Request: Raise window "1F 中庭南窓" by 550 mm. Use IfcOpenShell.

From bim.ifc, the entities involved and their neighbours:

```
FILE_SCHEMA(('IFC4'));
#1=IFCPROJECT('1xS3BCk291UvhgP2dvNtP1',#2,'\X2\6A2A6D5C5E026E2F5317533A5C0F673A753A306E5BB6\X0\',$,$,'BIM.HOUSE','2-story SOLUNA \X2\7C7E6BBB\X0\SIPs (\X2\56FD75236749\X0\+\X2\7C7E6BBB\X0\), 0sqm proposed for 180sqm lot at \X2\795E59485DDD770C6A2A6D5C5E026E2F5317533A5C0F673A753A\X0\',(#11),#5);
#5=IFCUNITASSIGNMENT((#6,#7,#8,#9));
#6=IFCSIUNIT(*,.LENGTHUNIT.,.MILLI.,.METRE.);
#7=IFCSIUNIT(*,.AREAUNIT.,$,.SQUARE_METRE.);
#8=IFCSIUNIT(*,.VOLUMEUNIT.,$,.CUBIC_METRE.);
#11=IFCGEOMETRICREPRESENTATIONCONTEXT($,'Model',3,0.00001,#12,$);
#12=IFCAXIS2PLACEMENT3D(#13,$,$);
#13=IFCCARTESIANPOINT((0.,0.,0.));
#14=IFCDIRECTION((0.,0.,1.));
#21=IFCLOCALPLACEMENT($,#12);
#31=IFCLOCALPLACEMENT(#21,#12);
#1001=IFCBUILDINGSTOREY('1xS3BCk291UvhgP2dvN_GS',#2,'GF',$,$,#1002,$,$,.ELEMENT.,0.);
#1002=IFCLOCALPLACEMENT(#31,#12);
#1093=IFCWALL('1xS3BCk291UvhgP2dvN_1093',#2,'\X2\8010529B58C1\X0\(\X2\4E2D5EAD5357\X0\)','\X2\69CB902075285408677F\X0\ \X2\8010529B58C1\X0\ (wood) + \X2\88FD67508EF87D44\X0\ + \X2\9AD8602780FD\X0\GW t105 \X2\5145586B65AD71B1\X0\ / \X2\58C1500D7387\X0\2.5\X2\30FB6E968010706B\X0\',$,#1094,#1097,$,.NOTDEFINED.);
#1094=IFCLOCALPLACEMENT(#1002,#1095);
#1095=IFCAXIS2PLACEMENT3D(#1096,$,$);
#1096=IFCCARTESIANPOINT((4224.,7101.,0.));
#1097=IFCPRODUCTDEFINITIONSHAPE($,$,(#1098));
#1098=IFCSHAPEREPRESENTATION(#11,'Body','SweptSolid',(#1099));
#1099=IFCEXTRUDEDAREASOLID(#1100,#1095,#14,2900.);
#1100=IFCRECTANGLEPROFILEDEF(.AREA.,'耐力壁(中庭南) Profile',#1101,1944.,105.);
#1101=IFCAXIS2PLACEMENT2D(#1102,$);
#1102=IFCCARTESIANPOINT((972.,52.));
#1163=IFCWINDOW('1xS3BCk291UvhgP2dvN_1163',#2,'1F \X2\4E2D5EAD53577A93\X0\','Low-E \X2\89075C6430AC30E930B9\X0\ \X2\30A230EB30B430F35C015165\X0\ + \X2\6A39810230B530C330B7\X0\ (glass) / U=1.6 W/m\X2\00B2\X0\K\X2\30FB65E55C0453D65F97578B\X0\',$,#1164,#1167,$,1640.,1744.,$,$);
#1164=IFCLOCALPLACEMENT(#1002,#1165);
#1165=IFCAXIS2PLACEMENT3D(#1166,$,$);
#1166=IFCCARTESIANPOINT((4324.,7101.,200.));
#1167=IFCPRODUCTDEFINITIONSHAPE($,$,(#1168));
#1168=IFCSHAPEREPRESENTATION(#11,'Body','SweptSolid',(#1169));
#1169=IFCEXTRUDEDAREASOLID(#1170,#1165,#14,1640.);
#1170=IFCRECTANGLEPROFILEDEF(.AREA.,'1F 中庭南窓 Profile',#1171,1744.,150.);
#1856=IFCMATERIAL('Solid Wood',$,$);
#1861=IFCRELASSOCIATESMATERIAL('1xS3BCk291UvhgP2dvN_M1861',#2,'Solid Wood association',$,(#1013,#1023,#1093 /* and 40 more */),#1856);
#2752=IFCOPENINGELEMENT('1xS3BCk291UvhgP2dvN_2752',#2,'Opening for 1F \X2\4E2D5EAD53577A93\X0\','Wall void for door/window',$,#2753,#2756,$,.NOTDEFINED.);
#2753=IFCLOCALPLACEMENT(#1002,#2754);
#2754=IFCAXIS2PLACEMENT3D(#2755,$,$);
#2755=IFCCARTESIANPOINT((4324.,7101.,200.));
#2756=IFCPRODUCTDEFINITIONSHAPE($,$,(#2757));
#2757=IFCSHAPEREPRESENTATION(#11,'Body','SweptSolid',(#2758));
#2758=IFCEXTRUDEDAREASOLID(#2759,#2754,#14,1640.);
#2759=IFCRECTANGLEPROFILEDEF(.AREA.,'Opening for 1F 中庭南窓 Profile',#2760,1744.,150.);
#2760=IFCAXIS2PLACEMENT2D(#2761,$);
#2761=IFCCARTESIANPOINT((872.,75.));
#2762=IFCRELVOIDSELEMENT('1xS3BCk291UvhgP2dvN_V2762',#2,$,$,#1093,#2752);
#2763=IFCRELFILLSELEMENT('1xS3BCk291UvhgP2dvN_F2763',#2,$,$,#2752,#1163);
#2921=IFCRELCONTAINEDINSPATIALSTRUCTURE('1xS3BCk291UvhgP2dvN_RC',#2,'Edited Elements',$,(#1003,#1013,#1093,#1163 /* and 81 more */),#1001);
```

```python
import numpy as np
import ifcopenshell
import ifcopenshell.api.geometry
import ifcopenshell.util.placement
import ifcopenshell.util.unit

model = ifcopenshell.open("bim.ifc")
unit_scale = ifcopenshell.util.unit.calculate_unit_scale(model)

window = model.by_guid("1xS3BCk291UvhgP2dvN_1163")
opening = window.FillsVoids[0].RelatingOpeningElement
dz = 0.55 / unit_scale

shift = np.array([0.0, 0.0, dz])
# The window is not placed relative to its opening, so move both.
for product in (opening, window):
    matrix = ifcopenshell.util.placement.get_local_placement(product.ObjectPlacement)
    matrix[:3, 3] += shift
    ifcopenshell.api.geometry.edit_object_placement(model, product=product, matrix=matrix, is_si=False)

print(f"moved by {dz * unit_scale:+.3f} m")

model.write("bim_updated.ifc")
```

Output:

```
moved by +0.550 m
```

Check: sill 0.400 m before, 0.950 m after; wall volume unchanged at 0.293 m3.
